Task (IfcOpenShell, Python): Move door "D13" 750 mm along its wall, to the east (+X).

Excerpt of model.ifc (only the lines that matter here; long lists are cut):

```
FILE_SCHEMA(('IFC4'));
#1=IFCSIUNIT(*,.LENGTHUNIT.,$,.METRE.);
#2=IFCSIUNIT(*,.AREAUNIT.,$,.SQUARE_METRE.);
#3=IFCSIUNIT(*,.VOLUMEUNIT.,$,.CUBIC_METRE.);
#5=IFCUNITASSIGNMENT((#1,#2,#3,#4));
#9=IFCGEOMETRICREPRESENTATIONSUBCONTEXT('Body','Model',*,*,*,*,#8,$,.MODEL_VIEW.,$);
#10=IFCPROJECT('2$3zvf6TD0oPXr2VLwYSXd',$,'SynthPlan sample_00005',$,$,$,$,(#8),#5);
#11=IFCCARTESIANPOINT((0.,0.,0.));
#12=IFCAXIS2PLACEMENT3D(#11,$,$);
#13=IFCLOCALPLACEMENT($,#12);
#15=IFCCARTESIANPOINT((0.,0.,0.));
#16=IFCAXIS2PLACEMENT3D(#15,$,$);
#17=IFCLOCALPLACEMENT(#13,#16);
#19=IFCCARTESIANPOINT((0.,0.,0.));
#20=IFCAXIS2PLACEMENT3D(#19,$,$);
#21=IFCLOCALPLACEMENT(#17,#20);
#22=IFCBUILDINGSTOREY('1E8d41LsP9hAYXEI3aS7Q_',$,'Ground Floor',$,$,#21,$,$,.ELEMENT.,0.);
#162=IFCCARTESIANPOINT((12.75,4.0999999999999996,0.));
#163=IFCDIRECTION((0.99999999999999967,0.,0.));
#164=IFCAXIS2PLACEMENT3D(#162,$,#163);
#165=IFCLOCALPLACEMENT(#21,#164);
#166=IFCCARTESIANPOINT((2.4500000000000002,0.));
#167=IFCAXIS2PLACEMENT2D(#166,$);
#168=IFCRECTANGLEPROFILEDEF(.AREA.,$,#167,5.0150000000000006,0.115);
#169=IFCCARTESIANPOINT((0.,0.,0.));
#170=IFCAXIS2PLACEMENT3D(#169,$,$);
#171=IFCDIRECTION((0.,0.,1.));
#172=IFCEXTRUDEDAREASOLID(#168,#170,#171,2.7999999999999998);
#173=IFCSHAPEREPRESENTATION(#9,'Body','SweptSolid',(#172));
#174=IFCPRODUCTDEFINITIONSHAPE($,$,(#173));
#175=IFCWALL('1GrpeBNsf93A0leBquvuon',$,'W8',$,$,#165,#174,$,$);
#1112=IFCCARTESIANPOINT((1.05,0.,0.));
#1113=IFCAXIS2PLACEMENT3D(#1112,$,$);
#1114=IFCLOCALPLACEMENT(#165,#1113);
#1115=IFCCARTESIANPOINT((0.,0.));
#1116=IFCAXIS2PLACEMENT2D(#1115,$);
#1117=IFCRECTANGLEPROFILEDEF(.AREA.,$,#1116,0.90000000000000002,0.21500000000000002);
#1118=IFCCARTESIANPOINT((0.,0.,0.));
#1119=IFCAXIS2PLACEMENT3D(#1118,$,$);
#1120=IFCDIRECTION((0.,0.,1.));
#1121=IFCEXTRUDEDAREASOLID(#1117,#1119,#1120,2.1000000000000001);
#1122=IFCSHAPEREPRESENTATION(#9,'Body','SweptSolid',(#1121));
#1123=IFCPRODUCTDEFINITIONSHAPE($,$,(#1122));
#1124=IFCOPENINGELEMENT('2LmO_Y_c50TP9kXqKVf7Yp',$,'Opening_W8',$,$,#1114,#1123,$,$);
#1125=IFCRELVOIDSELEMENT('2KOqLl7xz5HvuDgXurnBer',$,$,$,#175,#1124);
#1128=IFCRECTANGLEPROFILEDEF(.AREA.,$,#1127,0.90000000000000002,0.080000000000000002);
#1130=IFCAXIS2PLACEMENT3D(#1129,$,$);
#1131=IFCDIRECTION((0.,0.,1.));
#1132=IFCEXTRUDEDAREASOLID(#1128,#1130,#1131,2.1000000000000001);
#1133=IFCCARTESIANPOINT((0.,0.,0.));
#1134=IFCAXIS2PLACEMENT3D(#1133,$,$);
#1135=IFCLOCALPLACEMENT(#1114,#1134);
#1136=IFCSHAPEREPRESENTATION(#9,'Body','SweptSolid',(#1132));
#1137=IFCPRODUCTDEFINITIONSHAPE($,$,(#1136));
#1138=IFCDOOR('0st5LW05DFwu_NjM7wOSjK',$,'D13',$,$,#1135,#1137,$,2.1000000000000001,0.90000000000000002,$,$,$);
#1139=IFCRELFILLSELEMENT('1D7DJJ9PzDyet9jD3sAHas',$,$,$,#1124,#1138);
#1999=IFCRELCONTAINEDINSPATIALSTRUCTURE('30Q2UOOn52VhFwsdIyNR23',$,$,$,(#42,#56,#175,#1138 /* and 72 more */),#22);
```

```python
import ifcopenshell
import ifcopenshell.api.geometry
import ifcopenshell.util.placement

model = ifcopenshell.open("model.ifc")

door = model.by_guid("0st5LW05DFwu_NjM7wOSjK")
opening = door.FillsVoids[0].RelatingOpeningElement
wall = opening.VoidsElements[0].RelatingBuildingElement

wall_matrix = ifcopenshell.util.placement.get_local_placement(wall.ObjectPlacement)
shift = wall_matrix[:3, 0] * 0.75
before = ifcopenshell.util.placement.get_local_placement(door.ObjectPlacement)[:3, 3].copy()

# The door is placed relative to its opening, so it follows when the opening moves.
matrix = ifcopenshell.util.placement.get_local_placement(opening.ObjectPlacement)
matrix[:3, 3] += shift
ifcopenshell.api.geometry.edit_object_placement(
    model, product=opening, matrix=matrix, is_si=False, should_transform_children=True
)

after = ifcopenshell.util.placement.get_local_placement(door.ObjectPlacement)[:3, 3]
print("door moved by", (after - before).round(3) + 0.0)

model.write("model_rev.ifc")
```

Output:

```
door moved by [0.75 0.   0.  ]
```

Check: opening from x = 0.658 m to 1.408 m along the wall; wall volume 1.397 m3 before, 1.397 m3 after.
